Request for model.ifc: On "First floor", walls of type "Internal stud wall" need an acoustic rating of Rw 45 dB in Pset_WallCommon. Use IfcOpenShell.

First a look at what the model holds.

```python
import ifcopenshell
import ifcopenshell.util.element

model = ifcopenshell.open("model.ifc")
print(model.schema)
storey = next(s for s in model.by_type("IfcBuildingStorey") if s.Name == "First floor")
walls = [e for e in ifcopenshell.util.element.get_decomposition(storey) if e.is_a("IfcWall")]
seen = {}
for e in walls:
    element_type = ifcopenshell.util.element.get_type(e)
    key = (element_type.Name if element_type != e and element_type else None, ifcopenshell.util.element.get_pset(e, "Pset_WallCommon", "AcousticRating"))
    seen[key] = seen.get(key, 0) + 1
for (name, value), count in sorted(seen.items(), key=str):
    print(count, "x", name, "|", value)
```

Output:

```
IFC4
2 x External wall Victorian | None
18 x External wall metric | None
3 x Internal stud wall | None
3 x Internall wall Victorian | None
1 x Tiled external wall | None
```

```python
import ifcopenshell
import ifcopenshell.api.pset
import ifcopenshell.util.element

model = ifcopenshell.open("model.ifc")

storey = next(s for s in model.by_type("IfcBuildingStorey") if s.Name == "First floor")
walls = [e for e in ifcopenshell.util.element.get_decomposition(storey) if e.is_a("IfcWall")]

count = 0
for e in walls:
    element_type = ifcopenshell.util.element.get_type(e)
    if element_type in (None, e) or element_type.Name != "Internal stud wall":
        continue
    # add_pset returns the element's existing set when there is one.
    pset = ifcopenshell.api.pset.add_pset(model, product=e, name="Pset_WallCommon")
    ifcopenshell.api.pset.edit_pset(model, pset=pset, properties={"AcousticRating": "Rw 45 dB"})
    count += 1

print(count, "walls updated")

model.write("model-out.ifc")
```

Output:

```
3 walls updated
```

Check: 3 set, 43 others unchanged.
